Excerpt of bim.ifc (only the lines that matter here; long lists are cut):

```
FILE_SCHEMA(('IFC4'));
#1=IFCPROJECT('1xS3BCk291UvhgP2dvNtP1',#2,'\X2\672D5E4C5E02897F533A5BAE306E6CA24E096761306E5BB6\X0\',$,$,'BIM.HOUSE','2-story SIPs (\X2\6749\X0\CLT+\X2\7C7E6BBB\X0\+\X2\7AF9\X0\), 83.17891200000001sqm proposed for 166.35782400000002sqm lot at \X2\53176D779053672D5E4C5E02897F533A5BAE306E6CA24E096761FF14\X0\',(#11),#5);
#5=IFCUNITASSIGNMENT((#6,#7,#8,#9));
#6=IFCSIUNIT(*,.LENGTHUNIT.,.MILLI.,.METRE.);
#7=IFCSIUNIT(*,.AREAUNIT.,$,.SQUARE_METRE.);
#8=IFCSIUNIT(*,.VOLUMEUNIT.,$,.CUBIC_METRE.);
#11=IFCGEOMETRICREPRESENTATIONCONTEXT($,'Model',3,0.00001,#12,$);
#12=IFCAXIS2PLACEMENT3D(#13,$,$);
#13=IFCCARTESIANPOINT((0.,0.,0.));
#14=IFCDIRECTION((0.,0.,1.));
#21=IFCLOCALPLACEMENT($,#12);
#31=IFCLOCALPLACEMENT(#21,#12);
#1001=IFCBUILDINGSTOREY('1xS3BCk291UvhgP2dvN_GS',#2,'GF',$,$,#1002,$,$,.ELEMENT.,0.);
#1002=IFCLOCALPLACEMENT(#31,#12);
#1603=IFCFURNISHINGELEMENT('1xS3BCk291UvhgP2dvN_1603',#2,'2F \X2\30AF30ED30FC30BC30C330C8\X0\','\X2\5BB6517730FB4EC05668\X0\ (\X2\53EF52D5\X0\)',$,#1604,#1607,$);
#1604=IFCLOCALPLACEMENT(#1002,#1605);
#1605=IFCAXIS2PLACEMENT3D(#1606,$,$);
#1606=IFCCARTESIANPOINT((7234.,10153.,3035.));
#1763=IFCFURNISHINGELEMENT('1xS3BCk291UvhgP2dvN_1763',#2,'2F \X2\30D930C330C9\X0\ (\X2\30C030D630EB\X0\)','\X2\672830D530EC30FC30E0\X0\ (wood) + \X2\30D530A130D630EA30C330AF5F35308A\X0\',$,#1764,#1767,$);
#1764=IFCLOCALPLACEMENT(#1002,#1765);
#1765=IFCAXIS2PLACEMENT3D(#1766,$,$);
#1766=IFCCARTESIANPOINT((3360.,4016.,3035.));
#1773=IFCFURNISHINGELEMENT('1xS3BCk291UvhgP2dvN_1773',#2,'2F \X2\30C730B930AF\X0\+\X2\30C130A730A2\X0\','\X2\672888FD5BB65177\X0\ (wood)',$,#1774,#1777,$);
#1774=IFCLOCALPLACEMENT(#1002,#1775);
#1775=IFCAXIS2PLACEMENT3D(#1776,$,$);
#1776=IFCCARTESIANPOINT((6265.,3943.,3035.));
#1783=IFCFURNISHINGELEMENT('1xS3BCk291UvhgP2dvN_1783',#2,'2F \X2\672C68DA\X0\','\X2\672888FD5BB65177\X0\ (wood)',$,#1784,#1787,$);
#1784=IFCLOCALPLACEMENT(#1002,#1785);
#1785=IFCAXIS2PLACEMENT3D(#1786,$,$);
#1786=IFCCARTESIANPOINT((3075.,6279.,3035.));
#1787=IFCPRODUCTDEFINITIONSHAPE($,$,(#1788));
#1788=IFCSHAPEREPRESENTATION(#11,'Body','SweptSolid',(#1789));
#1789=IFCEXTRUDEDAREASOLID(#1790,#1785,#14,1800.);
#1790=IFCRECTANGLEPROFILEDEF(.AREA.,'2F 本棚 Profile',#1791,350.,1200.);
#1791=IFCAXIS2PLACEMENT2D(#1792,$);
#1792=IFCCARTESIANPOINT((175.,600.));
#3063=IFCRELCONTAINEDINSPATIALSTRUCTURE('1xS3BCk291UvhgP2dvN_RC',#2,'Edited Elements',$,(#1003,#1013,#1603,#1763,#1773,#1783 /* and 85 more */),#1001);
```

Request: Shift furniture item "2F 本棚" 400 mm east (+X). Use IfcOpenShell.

```python
import ifcopenshell
import ifcopenshell.api.geometry
import ifcopenshell.util.placement

model = ifcopenshell.open("bim.ifc")

item = model.by_guid("1xS3BCk291UvhgP2dvN_1783")
matrix = ifcopenshell.util.placement.get_local_placement(item.ObjectPlacement)
matrix[0, 3] += 400.0
ifcopenshell.api.geometry.edit_object_placement(model, product=item, matrix=matrix, is_si=False)

print(ifcopenshell.util.placement.get_local_placement(item.ObjectPlacement).round(3) + 0.0)

model.write("bim_rev.ifc")
```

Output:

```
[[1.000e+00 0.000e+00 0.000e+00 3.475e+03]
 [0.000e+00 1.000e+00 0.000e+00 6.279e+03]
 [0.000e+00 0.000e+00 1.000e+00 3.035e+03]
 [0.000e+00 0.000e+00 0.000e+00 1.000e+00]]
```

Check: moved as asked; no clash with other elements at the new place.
